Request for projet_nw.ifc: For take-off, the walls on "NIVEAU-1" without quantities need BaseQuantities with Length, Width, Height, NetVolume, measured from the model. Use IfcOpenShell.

First a look at what the model holds.

```python
import ifcopenshell
import ifcopenshell.util.element
import ifcopenshell.util.unit

model = ifcopenshell.open("projet_nw.ifc")
print(model.schema)
for unit_type in ("LENGTHUNIT", "AREAUNIT", "VOLUMEUNIT"):
    print(unit_type, ifcopenshell.util.unit.calculate_unit_scale(model, unit_type))
storey = next(s for s in model.by_type("IfcBuildingStorey") if s.Name == "NIVEAU-1")
walls = [e for e in ifcopenshell.util.element.get_decomposition(storey) if e.is_a("IfcWall")]
for e in sorted(walls, key=lambda e: e.id()):
    print(e.id(), e.is_a(), e.Name, list(ifcopenshell.util.element.get_psets(e, qtos_only=True)), sep=" | ")
```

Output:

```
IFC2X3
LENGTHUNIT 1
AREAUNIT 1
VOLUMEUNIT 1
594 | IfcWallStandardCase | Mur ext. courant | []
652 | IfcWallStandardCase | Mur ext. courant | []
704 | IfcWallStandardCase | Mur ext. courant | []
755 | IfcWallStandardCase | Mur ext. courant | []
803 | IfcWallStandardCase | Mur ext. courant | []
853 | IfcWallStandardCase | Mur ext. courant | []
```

```python
import ifcopenshell
import ifcopenshell.api.pset
import ifcopenshell.geom
import ifcopenshell.util.element
import ifcopenshell.util.shape
import ifcopenshell.util.unit

model = ifcopenshell.open("projet_nw.ifc")
unit_scale = ifcopenshell.util.unit.calculate_unit_scale(model)
volume_scale = ifcopenshell.util.unit.calculate_unit_scale(model, "VOLUMEUNIT")
settings = ifcopenshell.geom.settings()

storey = next(s for s in model.by_type("IfcBuildingStorey") if s.Name == "NIVEAU-1")
walls = [e for e in ifcopenshell.util.element.get_decomposition(storey) if e.is_a("IfcWall")]

for e in sorted(walls, key=lambda e: e.id()):
    if ifcopenshell.util.element.get_psets(e, qtos_only=True, should_inherit=False):
        continue
    # Geometry comes back in metres, in the element's own axes.
    shape = ifcopenshell.geom.create_shape(settings, e)
    values = {
        "Length": ifcopenshell.util.shape.get_x(shape.geometry) / unit_scale,
        "Width": ifcopenshell.util.shape.get_y(shape.geometry) / unit_scale,
        "Height": ifcopenshell.util.shape.get_z(shape.geometry) / unit_scale,
        "NetVolume": ifcopenshell.util.shape.get_volume(shape.geometry) / volume_scale,
    }
    qto = ifcopenshell.api.pset.add_qto(model, product=e, name="BaseQuantities")
    ifcopenshell.api.pset.edit_qto(model, qto=qto, properties=values)
    print(e.id(), {k: round(v, 3) for k, v in values.items()})

model.write("projet_nw_v2.ifc")
```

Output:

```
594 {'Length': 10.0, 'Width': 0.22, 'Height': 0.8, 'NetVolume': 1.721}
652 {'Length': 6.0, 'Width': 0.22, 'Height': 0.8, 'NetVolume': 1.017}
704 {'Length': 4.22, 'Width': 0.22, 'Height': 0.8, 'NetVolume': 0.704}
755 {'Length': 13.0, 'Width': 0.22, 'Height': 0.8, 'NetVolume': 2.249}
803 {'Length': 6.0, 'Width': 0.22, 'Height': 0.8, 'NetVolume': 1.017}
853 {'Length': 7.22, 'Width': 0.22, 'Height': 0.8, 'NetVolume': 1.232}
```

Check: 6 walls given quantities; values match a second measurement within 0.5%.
